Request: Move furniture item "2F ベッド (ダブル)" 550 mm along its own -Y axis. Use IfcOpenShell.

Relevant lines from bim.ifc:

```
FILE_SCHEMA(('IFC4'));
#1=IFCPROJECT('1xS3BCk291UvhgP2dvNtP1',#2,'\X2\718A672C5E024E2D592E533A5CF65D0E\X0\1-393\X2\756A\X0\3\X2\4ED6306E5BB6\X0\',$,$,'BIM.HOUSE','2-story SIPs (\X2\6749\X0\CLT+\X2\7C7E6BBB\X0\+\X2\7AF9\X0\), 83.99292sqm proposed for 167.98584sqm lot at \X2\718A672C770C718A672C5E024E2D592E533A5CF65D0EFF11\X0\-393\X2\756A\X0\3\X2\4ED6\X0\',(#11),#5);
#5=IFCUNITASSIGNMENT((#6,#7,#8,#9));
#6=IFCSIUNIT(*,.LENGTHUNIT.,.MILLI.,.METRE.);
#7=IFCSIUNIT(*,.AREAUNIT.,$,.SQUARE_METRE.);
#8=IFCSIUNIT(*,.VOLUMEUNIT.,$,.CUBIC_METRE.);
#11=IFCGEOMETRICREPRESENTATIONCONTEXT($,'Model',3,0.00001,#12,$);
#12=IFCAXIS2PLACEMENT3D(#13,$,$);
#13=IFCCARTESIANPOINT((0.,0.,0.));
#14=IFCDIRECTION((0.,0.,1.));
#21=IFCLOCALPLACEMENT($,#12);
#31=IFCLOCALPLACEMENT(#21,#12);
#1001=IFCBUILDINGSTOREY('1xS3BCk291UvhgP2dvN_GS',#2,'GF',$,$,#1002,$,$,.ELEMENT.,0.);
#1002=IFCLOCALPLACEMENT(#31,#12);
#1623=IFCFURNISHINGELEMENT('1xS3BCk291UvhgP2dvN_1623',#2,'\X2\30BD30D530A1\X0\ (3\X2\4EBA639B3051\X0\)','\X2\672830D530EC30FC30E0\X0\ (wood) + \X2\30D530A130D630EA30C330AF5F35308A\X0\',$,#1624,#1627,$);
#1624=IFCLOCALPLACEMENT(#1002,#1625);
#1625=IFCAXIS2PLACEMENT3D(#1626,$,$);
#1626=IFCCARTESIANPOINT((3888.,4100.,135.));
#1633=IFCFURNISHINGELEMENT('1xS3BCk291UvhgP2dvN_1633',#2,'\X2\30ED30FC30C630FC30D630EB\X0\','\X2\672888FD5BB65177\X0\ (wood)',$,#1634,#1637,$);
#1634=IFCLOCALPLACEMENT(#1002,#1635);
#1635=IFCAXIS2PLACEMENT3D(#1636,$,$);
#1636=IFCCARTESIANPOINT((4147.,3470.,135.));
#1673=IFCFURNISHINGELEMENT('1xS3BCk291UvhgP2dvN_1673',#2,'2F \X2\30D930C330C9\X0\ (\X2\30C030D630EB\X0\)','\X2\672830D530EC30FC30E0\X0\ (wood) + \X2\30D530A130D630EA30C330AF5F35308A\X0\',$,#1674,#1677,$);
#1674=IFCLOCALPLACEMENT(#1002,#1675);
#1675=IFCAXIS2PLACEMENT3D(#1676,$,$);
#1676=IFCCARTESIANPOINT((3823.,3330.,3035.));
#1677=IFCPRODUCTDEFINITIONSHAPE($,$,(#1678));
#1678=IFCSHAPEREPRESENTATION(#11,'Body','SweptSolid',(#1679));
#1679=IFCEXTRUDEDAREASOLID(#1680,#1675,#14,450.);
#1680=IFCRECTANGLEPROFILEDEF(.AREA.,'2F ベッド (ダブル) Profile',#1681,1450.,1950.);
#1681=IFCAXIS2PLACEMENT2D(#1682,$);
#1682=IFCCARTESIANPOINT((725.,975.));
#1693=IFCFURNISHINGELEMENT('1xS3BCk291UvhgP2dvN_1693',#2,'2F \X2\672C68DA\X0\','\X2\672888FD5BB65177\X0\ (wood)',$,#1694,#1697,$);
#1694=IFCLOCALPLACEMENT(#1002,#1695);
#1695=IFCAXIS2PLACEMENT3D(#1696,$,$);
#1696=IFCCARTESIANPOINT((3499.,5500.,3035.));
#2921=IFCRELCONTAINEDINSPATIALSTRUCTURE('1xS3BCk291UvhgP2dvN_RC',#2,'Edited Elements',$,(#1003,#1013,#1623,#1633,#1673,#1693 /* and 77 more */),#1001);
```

```python
import ifcopenshell
import ifcopenshell.api.geometry
import ifcopenshell.util.placement
import ifcopenshell.util.unit

model = ifcopenshell.open("bim.ifc")
unit_scale = ifcopenshell.util.unit.calculate_unit_scale(model)

item = model.by_guid("1xS3BCk291UvhgP2dvN_1673")
matrix = ifcopenshell.util.placement.get_local_placement(item.ObjectPlacement)
matrix[:3, 3] -= matrix[:3, 1] * 0.55 / unit_scale
ifcopenshell.api.geometry.edit_object_placement(model, product=item, matrix=matrix, is_si=False)

print(ifcopenshell.util.placement.get_local_placement(item.ObjectPlacement).round(3) + 0.0)

model.write("bim-out.ifc")
```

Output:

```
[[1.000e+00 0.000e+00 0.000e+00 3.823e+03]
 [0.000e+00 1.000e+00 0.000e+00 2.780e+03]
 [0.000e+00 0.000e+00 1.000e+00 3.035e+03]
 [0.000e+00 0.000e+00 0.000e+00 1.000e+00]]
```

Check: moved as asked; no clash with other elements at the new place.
